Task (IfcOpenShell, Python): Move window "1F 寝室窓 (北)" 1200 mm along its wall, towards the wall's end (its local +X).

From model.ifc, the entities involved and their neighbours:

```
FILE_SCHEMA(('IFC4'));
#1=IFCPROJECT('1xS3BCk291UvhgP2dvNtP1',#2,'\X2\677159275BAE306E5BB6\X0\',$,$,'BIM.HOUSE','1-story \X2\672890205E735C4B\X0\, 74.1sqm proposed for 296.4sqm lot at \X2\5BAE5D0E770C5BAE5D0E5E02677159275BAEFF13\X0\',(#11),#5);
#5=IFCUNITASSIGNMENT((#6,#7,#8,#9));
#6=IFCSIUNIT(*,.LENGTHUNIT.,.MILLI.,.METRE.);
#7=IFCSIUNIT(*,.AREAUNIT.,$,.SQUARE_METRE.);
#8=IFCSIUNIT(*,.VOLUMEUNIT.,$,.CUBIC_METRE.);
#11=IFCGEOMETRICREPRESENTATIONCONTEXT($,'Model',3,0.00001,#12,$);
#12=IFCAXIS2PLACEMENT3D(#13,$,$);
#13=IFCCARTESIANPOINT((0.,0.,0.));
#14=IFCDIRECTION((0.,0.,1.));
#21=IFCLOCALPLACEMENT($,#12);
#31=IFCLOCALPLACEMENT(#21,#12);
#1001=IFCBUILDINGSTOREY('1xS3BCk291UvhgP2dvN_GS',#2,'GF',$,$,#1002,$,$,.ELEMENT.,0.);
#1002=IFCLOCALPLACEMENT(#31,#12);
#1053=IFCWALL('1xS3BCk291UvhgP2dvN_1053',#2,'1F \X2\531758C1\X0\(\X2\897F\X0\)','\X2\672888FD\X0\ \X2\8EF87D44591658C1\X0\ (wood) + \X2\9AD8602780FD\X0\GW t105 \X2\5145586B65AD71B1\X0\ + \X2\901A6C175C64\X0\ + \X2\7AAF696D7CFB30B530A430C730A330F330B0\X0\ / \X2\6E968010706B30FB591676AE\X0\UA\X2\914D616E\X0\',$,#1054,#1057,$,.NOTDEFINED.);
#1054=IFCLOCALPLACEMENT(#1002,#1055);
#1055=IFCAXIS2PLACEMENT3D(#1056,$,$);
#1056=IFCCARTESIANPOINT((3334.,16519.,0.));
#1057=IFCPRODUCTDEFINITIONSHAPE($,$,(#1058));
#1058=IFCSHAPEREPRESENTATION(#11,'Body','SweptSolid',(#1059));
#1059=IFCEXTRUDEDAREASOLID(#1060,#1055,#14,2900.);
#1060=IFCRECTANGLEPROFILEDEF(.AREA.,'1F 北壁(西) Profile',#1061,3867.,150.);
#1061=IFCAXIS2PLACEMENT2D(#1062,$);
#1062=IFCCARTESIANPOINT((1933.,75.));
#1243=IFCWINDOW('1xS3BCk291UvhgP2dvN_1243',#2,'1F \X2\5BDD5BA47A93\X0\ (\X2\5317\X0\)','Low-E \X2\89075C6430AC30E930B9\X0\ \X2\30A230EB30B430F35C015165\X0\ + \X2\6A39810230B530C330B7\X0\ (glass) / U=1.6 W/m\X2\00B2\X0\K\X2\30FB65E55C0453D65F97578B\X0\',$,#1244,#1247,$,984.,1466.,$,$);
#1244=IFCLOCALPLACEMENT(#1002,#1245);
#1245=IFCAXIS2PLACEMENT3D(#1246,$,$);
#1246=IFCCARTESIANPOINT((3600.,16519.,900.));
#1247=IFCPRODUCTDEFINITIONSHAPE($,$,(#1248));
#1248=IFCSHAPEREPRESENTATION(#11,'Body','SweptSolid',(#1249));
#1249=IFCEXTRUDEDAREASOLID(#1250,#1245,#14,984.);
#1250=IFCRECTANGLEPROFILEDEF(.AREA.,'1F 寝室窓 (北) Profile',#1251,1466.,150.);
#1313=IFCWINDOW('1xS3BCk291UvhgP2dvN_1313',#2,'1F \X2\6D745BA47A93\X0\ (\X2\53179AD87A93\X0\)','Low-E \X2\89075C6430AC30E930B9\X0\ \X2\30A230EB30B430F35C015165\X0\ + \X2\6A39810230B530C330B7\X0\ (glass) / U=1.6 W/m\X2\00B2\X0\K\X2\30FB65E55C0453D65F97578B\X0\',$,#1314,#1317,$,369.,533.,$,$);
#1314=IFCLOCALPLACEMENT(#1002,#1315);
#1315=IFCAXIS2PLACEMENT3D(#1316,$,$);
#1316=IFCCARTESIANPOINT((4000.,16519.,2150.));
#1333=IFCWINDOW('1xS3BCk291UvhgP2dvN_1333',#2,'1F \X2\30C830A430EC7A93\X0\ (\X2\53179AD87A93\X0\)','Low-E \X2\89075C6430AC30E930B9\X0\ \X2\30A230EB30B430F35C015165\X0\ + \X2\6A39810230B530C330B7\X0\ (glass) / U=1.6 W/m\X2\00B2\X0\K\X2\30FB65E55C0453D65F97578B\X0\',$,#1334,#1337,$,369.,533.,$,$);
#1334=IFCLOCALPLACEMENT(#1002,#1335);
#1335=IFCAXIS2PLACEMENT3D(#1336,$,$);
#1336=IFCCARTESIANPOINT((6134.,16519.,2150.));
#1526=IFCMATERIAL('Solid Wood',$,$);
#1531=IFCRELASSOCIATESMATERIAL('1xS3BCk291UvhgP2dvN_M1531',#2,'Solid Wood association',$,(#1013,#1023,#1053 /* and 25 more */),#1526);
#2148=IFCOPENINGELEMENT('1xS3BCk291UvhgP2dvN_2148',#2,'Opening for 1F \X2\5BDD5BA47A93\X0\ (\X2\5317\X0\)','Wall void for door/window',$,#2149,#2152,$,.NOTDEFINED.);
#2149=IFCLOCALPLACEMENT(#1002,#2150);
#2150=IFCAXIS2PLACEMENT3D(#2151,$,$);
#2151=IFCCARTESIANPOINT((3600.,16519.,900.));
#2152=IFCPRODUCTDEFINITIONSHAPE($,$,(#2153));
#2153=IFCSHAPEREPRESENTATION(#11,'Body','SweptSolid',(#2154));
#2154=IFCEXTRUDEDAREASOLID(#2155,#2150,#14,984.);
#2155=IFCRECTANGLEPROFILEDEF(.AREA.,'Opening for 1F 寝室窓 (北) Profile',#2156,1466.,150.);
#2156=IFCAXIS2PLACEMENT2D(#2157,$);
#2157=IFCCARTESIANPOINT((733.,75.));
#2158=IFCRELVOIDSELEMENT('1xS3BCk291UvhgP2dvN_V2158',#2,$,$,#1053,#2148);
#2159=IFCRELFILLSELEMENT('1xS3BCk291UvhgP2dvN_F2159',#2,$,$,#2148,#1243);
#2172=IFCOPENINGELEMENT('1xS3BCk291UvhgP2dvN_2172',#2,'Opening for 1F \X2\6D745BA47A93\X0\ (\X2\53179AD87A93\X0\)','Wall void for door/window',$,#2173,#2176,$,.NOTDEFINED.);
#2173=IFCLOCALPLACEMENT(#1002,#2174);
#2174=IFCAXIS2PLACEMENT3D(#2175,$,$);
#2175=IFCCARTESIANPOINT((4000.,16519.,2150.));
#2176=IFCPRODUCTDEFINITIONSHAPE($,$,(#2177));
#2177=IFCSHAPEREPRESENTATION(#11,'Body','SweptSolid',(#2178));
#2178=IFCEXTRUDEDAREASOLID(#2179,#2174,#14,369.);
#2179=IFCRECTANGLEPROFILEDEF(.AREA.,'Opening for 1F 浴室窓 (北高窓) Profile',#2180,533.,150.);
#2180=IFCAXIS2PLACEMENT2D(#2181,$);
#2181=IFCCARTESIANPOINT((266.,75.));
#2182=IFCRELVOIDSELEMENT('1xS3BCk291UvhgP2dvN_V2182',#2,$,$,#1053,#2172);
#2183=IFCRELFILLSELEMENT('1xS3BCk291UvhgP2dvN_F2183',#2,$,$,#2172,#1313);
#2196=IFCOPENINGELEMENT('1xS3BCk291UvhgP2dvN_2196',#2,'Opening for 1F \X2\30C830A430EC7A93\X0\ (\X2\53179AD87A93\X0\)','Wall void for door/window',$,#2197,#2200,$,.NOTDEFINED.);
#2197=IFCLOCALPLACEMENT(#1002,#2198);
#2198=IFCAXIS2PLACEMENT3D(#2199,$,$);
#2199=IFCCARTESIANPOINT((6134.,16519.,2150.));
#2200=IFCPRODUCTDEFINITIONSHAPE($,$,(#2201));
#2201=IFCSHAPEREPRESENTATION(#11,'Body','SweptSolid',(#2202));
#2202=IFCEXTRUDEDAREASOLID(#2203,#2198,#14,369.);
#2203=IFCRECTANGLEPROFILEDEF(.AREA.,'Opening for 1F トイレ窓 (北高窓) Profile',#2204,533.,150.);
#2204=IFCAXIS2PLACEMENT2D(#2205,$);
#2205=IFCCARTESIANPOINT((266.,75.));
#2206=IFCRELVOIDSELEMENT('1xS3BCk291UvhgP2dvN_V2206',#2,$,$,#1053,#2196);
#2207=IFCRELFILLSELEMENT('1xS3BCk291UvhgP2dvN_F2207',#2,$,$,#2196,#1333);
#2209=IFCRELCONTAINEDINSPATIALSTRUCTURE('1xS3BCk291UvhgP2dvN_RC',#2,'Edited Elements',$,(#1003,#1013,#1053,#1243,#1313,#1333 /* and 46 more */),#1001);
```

```python
import ifcopenshell
import ifcopenshell.api.geometry
import ifcopenshell.util.placement

model = ifcopenshell.open("model.ifc")

window = model.by_guid("1xS3BCk291UvhgP2dvN_1243")
opening = window.FillsVoids[0].RelatingOpeningElement
wall = opening.VoidsElements[0].RelatingBuildingElement

wall_matrix = ifcopenshell.util.placement.get_local_placement(wall.ObjectPlacement)
shift = wall_matrix[:3, 0] * 1200.0
before = ifcopenshell.util.placement.get_local_placement(window.ObjectPlacement)[:3, 3].copy()

# The window is not placed relative to its opening, so move both.
for product in (opening, window):
    matrix = ifcopenshell.util.placement.get_local_placement(product.ObjectPlacement)
    matrix[:3, 3] += shift
    ifcopenshell.api.geometry.edit_object_placement(model, product=product, matrix=matrix, is_si=False)

after = ifcopenshell.util.placement.get_local_placement(window.ObjectPlacement)[:3, 3]
print("window moved by", (after - before).round(3) + 0.0)

model.write("model_updated.ifc")
```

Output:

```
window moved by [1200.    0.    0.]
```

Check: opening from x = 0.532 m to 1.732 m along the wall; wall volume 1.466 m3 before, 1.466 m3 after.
